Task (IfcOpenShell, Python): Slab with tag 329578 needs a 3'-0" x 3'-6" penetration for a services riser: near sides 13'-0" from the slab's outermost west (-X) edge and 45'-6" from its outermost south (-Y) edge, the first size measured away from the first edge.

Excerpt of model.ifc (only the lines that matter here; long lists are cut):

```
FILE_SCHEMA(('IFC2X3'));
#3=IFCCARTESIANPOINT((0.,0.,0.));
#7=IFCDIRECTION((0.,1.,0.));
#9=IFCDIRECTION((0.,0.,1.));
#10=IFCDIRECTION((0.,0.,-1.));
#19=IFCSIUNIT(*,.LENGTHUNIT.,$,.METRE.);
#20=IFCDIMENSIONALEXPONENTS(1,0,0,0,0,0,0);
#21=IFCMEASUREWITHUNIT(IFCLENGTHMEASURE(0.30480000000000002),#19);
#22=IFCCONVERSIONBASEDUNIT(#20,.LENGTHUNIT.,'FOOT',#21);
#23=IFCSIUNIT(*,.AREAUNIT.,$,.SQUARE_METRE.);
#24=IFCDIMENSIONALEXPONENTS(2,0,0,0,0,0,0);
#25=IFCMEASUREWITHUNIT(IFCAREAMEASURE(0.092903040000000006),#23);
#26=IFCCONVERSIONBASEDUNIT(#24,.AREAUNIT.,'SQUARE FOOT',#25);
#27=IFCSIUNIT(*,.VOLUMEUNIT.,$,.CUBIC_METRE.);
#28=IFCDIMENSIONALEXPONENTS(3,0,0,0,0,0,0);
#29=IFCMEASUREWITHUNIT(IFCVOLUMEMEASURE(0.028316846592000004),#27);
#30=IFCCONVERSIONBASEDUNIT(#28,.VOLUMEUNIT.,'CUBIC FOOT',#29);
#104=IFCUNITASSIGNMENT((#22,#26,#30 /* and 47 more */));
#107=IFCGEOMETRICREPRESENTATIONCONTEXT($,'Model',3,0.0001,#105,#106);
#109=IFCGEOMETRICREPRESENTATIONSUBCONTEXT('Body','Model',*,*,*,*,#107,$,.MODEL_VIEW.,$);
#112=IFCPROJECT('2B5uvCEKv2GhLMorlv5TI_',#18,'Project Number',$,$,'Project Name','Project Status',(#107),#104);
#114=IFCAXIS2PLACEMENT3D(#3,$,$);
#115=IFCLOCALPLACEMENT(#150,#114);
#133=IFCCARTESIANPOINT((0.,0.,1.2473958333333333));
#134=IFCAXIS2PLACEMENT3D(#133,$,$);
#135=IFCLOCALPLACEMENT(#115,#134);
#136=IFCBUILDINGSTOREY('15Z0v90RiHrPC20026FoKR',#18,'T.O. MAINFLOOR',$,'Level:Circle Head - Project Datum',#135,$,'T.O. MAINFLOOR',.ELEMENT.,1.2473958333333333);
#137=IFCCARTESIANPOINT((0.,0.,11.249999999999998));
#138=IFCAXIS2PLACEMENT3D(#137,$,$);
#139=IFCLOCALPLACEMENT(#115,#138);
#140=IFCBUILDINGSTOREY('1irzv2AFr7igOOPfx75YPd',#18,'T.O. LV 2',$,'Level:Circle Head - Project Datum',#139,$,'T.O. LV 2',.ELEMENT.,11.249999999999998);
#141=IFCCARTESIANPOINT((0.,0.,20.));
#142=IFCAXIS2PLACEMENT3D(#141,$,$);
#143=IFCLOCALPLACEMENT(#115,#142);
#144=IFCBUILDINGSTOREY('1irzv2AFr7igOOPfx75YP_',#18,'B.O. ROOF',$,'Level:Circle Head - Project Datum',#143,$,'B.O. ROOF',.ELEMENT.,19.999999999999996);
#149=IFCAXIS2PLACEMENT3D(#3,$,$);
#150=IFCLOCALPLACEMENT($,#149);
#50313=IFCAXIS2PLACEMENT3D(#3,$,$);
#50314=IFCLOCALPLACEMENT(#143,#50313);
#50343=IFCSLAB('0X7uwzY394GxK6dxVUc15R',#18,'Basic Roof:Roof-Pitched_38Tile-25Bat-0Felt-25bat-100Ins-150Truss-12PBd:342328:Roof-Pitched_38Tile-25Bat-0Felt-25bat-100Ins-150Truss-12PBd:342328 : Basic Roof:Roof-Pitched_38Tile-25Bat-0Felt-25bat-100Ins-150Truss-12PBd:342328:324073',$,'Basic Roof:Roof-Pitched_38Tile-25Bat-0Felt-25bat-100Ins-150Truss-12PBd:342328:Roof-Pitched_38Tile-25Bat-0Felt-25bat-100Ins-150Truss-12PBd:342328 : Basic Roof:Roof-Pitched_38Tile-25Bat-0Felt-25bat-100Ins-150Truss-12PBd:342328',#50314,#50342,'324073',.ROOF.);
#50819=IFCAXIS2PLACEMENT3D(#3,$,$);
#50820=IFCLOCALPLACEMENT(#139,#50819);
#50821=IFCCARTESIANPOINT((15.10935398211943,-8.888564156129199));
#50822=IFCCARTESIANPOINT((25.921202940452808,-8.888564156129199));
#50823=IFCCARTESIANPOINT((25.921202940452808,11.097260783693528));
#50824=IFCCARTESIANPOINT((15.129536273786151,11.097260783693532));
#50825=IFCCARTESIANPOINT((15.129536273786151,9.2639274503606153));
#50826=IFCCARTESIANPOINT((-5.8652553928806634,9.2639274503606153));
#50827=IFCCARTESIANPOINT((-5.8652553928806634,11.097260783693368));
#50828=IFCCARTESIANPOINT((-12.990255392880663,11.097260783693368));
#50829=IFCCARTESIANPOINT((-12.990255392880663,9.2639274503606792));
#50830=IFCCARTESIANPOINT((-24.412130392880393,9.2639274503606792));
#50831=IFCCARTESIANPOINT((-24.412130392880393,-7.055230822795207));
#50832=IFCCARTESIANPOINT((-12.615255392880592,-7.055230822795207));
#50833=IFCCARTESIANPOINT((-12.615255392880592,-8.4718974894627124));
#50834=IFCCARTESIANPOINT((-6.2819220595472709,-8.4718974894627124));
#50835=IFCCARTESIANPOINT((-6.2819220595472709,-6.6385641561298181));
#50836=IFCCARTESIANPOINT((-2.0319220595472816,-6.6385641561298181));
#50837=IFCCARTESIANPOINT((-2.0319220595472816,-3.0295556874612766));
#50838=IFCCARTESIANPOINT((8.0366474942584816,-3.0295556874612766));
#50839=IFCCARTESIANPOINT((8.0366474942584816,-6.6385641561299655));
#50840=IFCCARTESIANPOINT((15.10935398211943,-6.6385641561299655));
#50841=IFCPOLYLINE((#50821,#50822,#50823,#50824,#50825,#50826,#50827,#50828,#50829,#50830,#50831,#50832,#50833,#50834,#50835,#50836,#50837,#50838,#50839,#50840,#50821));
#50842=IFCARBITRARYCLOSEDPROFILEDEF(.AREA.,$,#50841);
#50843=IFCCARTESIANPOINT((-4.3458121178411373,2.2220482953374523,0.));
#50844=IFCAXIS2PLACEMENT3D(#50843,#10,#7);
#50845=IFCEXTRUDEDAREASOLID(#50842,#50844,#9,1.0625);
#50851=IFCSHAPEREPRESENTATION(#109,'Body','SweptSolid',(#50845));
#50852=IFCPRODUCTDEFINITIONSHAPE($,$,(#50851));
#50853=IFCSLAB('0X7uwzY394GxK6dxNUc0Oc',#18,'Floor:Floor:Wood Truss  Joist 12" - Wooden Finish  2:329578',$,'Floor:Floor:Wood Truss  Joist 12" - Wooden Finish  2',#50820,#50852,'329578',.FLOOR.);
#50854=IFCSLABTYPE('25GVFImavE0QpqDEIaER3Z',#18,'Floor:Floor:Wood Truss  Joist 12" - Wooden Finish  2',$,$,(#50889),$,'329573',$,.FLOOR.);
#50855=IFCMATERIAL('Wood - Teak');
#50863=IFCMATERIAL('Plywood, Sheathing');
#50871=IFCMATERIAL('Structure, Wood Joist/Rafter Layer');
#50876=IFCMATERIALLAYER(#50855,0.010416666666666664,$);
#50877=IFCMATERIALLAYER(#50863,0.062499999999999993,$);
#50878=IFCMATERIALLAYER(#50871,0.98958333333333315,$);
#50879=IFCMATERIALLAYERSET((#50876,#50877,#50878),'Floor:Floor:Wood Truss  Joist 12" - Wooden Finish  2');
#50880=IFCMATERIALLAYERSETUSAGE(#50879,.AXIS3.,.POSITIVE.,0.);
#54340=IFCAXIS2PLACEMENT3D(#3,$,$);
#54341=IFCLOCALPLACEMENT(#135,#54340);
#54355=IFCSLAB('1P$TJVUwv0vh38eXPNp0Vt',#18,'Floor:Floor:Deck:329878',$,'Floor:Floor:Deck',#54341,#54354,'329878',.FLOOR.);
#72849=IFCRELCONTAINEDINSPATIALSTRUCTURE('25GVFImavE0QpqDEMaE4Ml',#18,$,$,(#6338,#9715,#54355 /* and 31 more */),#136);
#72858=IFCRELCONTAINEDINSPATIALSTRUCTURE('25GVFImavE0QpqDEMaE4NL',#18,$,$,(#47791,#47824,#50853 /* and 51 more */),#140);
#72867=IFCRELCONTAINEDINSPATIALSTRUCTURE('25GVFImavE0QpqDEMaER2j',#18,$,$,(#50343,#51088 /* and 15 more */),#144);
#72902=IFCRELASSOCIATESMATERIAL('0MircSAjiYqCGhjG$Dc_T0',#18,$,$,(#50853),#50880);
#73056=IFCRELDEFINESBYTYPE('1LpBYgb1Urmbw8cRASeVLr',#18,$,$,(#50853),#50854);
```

```python
import numpy as np
import ifcopenshell
import ifcopenshell.api.feature
import ifcopenshell.api.geometry
import ifcopenshell.api.root
import ifcopenshell.geom
import ifcopenshell.util.placement
import ifcopenshell.util.representation
import ifcopenshell.util.shape
import ifcopenshell.util.unit

model = ifcopenshell.open("model.ifc")
unit_scale = ifcopenshell.util.unit.calculate_unit_scale(model)
settings = ifcopenshell.geom.settings()


def volume(element):
    """Net volume in cubic metres, openings subtracted."""
    shape = ifcopenshell.geom.create_shape(settings, element)
    return ifcopenshell.util.shape.get_volume(shape.geometry)


slab = model.by_id(50853)
before = volume(slab)

# Extent in the slab's own axes, in metres. The edges named are its -X and -Y sides.
slab_shape = ifcopenshell.geom.create_shape(settings, slab)
vertices = ifcopenshell.util.shape.get_vertices(slab_shape.geometry)
x_min, y_min, bottom = vertices.min(axis=0)
top = vertices[:, 2].max()

opening = ifcopenshell.api.root.create_entity(model, ifc_class="IfcOpeningElement", name="Services riser opening")
context = ifcopenshell.util.representation.get_context(model, "Model", "Body", "MODEL_VIEW")
width, depth = 0.9144, 1.0668
outline = [(0.0, 0.0), (width, 0.0), (width, depth), (0.0, depth), (0.0, 0.0)]
# Overshoot both faces by 50 mm so the cut is clean.
shape = ifcopenshell.api.geometry.add_slab_representation(
    model, context=context, depth=top - bottom + 0.1, polyline=outline
)
ifcopenshell.api.geometry.assign_representation(model, product=opening, representation=shape)

matrix = ifcopenshell.util.placement.get_local_placement(slab.ObjectPlacement)
matrix[:, 3] = matrix @ np.append(np.array([x_min + 3.9624, y_min + 13.8684, bottom - 0.05]) / unit_scale, 1.0)
ifcopenshell.api.geometry.edit_object_placement(model, product=opening, matrix=matrix, is_si=False)
ifcopenshell.api.feature.add_feature(model, feature=opening, element=slab)

after = volume(slab)

print(f"slab volume {before:.3f} -> {after:.3f} m3")

model.write("model-out.ifc")
```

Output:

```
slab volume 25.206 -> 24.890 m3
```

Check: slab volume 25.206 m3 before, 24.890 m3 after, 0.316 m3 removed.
